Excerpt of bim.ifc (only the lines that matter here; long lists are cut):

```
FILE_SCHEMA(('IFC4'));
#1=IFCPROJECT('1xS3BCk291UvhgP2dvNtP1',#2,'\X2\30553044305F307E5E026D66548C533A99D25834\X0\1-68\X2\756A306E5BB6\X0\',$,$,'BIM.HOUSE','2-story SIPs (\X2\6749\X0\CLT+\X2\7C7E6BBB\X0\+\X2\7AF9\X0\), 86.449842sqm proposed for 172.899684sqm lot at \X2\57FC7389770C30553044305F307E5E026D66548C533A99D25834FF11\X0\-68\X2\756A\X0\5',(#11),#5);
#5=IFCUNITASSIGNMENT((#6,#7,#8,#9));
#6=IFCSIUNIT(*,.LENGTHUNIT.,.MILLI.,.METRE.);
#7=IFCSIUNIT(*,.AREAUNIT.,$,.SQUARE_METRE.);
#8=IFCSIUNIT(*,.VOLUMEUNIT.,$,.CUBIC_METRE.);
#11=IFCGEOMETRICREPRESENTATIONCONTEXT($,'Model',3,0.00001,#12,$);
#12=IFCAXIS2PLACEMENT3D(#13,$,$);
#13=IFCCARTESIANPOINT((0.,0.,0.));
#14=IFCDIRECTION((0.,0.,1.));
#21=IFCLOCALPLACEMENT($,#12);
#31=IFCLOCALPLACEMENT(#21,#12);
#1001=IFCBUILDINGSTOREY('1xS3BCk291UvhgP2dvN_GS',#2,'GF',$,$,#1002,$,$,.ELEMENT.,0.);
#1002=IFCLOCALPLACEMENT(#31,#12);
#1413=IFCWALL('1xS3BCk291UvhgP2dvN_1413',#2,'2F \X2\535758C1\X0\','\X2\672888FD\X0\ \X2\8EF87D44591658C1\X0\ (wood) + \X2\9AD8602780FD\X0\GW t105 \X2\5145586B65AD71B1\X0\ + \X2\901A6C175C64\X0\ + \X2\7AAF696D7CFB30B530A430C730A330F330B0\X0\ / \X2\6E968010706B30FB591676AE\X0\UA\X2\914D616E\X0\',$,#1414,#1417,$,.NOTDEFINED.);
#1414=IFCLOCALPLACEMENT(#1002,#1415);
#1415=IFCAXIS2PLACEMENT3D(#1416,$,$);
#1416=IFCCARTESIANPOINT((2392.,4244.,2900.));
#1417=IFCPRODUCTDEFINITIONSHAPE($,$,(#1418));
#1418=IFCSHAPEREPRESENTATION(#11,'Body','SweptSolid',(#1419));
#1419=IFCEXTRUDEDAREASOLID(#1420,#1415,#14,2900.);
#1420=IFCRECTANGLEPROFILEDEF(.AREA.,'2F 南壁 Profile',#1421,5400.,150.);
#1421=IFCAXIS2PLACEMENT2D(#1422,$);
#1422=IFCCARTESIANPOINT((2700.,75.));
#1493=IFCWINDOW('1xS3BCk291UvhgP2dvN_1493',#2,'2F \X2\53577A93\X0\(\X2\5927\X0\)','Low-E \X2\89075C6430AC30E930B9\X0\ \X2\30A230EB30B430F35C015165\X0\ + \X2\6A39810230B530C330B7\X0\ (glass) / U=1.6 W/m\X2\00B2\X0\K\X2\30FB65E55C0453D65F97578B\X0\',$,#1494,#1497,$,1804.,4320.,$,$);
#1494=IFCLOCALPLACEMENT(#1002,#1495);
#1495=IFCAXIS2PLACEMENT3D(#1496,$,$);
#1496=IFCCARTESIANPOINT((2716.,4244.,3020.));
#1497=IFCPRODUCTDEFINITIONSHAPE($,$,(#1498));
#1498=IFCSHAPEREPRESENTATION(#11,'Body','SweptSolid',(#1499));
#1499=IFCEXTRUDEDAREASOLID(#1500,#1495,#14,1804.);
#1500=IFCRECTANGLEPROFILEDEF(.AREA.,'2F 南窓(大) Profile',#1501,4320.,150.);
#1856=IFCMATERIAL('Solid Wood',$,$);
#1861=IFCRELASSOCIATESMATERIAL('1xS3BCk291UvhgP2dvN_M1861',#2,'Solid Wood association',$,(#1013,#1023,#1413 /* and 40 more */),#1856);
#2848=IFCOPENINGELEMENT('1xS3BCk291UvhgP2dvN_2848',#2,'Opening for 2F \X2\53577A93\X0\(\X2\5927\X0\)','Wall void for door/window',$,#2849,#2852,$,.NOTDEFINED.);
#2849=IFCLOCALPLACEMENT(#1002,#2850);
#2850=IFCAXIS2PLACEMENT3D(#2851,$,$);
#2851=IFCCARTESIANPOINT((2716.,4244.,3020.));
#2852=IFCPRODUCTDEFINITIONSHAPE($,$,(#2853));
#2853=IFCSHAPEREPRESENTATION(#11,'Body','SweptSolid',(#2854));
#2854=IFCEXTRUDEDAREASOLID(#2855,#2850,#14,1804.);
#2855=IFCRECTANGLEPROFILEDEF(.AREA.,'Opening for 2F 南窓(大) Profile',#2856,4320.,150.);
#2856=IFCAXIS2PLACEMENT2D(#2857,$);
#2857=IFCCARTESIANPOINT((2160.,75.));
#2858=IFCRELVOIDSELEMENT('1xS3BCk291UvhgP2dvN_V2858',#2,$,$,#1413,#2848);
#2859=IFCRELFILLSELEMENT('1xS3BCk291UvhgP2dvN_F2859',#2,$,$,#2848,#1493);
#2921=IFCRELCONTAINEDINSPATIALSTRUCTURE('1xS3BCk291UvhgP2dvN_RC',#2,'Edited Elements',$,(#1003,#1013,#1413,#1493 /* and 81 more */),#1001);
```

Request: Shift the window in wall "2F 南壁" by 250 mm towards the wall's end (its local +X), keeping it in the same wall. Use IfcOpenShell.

```python
import ifcopenshell
import ifcopenshell.api.geometry
import ifcopenshell.util.placement
import ifcopenshell.util.unit

model = ifcopenshell.open("bim.ifc")
unit_scale = ifcopenshell.util.unit.calculate_unit_scale(model)

window = model.by_guid("1xS3BCk291UvhgP2dvN_1493")
opening = window.FillsVoids[0].RelatingOpeningElement
wall = opening.VoidsElements[0].RelatingBuildingElement

wall_matrix = ifcopenshell.util.placement.get_local_placement(wall.ObjectPlacement)
shift = wall_matrix[:3, 0] * 0.25 / unit_scale
before = ifcopenshell.util.placement.get_local_placement(window.ObjectPlacement)[:3, 3].copy()

# The window is not placed relative to its opening, so move both.
for product in (opening, window):
    matrix = ifcopenshell.util.placement.get_local_placement(product.ObjectPlacement)
    matrix[:3, 3] += shift
    ifcopenshell.api.geometry.edit_object_placement(model, product=product, matrix=matrix, is_si=False)

after = ifcopenshell.util.placement.get_local_placement(window.ObjectPlacement)[:3, 3]
print("window moved by", (after - before).round(3) + 0.0)

model.write("bim-out.ifc")
```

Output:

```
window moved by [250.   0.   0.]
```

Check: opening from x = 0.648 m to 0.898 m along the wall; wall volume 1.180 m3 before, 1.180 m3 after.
